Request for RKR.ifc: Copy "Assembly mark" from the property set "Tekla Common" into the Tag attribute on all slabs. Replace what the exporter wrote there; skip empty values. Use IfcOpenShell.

First a look at what the model holds.

```python
import ifcopenshell
import ifcopenshell.util.element

model = ifcopenshell.open("RKR.ifc")
print(model.schema)
slabs = model.by_type("IfcSlab")
print(len(slabs), "slabs")
for e in slabs[:8]:
    source = ifcopenshell.util.element.get_pset(e, "Tekla Common", "Assembly mark")
    target = e.Tag
    print(e.id(), repr(source), repr(target), sep=" | ")
```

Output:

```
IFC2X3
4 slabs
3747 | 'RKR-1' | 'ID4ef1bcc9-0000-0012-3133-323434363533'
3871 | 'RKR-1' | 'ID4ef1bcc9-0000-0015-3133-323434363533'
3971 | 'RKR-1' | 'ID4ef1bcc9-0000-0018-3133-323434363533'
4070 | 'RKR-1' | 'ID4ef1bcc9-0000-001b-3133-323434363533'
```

```python
import ifcopenshell
import ifcopenshell.util.element

model = ifcopenshell.open("RKR.ifc")

count = 0
for e in model.by_type("IfcSlab"):
    value = ifcopenshell.util.element.get_pset(e, "Tekla Common", "Assembly mark")
    current = e.Tag
    if not value or not value.strip() or current == value:
        continue
    e.Tag = value
    count += 1

print(count, "slabs updated")

model.write("RKR_updated.ifc")
```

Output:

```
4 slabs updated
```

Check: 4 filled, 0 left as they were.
